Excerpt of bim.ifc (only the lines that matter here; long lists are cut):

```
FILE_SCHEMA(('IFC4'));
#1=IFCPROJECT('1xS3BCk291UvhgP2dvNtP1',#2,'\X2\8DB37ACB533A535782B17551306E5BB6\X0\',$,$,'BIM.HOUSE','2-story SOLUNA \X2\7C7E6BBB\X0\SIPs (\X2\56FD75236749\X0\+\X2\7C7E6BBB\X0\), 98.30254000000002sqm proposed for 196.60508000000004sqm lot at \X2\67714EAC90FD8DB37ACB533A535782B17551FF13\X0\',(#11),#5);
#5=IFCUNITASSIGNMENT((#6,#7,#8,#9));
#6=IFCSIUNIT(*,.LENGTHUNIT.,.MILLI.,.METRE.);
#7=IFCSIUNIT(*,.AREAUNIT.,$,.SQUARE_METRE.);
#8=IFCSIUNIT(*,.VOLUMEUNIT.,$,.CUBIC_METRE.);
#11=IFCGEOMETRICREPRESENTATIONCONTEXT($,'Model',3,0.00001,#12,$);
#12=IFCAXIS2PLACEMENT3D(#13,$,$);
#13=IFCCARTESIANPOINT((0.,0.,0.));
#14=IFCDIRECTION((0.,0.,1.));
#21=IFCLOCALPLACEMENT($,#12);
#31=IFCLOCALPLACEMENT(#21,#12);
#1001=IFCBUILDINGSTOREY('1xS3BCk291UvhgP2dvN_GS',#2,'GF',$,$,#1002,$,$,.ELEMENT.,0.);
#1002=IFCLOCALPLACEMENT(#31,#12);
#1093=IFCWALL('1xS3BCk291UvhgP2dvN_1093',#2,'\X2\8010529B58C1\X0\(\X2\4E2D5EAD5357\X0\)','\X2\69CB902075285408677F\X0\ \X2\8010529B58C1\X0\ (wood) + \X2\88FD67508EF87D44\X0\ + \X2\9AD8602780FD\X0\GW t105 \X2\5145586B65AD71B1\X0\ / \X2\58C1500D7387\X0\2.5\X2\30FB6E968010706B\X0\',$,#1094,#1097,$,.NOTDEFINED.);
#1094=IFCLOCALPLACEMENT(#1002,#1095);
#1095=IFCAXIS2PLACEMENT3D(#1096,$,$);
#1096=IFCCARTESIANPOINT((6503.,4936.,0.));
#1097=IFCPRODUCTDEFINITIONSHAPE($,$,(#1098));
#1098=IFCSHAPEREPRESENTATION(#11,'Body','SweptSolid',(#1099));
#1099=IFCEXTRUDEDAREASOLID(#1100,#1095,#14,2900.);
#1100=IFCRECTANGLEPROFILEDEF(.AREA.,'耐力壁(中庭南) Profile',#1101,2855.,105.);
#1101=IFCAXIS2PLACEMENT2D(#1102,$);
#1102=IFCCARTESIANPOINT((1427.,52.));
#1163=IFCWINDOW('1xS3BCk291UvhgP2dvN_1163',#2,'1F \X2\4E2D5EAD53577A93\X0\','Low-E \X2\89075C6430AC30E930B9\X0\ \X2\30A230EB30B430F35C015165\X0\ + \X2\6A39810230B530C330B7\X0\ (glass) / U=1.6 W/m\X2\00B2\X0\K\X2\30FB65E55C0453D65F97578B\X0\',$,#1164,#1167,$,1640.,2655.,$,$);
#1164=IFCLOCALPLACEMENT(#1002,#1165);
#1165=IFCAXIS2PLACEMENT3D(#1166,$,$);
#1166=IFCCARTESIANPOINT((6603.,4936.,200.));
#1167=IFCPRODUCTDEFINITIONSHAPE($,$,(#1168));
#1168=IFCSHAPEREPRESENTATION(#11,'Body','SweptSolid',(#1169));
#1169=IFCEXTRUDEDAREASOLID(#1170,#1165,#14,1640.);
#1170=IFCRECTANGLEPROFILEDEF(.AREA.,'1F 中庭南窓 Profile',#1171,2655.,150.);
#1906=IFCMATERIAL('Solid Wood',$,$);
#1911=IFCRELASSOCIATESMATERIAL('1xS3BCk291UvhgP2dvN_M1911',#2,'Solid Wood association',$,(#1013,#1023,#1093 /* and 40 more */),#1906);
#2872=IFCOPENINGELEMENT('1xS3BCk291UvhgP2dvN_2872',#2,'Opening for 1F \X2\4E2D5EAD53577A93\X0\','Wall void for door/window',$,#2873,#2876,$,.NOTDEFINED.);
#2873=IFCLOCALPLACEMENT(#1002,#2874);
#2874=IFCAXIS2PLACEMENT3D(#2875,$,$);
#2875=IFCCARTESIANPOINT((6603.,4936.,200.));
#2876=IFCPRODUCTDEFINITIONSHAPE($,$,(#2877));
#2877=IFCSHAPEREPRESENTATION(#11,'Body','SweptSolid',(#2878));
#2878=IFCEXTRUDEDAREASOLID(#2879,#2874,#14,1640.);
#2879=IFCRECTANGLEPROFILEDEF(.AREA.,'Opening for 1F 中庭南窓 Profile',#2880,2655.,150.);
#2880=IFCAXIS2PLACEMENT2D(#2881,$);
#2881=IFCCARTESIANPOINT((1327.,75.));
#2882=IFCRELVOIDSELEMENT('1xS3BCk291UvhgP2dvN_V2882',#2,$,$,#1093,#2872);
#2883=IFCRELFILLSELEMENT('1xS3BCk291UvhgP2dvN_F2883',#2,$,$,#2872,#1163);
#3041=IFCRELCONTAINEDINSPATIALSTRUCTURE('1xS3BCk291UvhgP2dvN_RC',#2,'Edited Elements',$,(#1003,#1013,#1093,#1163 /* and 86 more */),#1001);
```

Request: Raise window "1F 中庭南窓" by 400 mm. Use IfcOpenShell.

```python
import numpy as np
import ifcopenshell
import ifcopenshell.api.geometry
import ifcopenshell.util.placement
import ifcopenshell.util.unit

model = ifcopenshell.open("bim.ifc")
unit_scale = ifcopenshell.util.unit.calculate_unit_scale(model)

window = model.by_guid("1xS3BCk291UvhgP2dvN_1163")
opening = window.FillsVoids[0].RelatingOpeningElement
dz = 0.4 / unit_scale

shift = np.array([0.0, 0.0, dz])
# The window is not placed relative to its opening, so move both.
for product in (opening, window):
    matrix = ifcopenshell.util.placement.get_local_placement(product.ObjectPlacement)
    matrix[:3, 3] += shift
    ifcopenshell.api.geometry.edit_object_placement(model, product=product, matrix=matrix, is_si=False)

print(f"moved by {dz * unit_scale:+.3f} m")

model.write("bim_v2.ifc")
```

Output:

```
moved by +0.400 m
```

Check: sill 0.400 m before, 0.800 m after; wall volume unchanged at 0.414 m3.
